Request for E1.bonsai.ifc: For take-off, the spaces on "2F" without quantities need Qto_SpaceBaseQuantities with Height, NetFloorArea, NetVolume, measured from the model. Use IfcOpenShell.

First a look at what the model holds.

```python
import ifcopenshell
import ifcopenshell.util.element
import ifcopenshell.util.unit

model = ifcopenshell.open("E1.bonsai.ifc")
print(model.schema)
for unit_type in ("LENGTHUNIT", "AREAUNIT", "VOLUMEUNIT"):
    print(unit_type, ifcopenshell.util.unit.calculate_unit_scale(model, unit_type))
storey = next(s for s in model.by_type("IfcBuildingStorey") if s.Name == "2F")
spaces = [e for e in ifcopenshell.util.element.get_decomposition(storey) if e.is_a("IfcSpace")]
for e in sorted(spaces, key=lambda e: e.id()):
    print(e.id(), e.is_a(), e.Name, list(ifcopenshell.util.element.get_psets(e, qtos_only=True)), sep=" | ")
```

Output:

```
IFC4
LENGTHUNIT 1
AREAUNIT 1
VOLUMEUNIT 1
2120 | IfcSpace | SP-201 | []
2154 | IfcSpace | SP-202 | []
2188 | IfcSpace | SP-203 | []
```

```python
import ifcopenshell
import ifcopenshell.api.pset
import ifcopenshell.geom
import ifcopenshell.util.element
import ifcopenshell.util.shape
import ifcopenshell.util.unit

model = ifcopenshell.open("E1.bonsai.ifc")
unit_scale = ifcopenshell.util.unit.calculate_unit_scale(model)
area_scale = ifcopenshell.util.unit.calculate_unit_scale(model, "AREAUNIT")
volume_scale = ifcopenshell.util.unit.calculate_unit_scale(model, "VOLUMEUNIT")
settings = ifcopenshell.geom.settings()

storey = next(s for s in model.by_type("IfcBuildingStorey") if s.Name == "2F")
spaces = [e for e in ifcopenshell.util.element.get_decomposition(storey) if e.is_a("IfcSpace")]

for e in sorted(spaces, key=lambda e: e.id()):
    if ifcopenshell.util.element.get_psets(e, qtos_only=True, should_inherit=False):
        continue
    # Geometry comes back in metres, in the element's own axes.
    shape = ifcopenshell.geom.create_shape(settings, e)
    values = {
        "Height": ifcopenshell.util.shape.get_z(shape.geometry) / unit_scale,
        "NetFloorArea": ifcopenshell.util.shape.get_footprint_area(shape.geometry) / area_scale,
        "NetVolume": ifcopenshell.util.shape.get_volume(shape.geometry) / volume_scale,
    }
    qto = ifcopenshell.api.pset.add_qto(model, product=e, name="Qto_SpaceBaseQuantities")
    ifcopenshell.api.pset.edit_qto(model, qto=qto, properties=values)
    print(e.id(), {k: round(v, 3) for k, v in values.items()})

model.write("E1.bonsai_v2.ifc")
```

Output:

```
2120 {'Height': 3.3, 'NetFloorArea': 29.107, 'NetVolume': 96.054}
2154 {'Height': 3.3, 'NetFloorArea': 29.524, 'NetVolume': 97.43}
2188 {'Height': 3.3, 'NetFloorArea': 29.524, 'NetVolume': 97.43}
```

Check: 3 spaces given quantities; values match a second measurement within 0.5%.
